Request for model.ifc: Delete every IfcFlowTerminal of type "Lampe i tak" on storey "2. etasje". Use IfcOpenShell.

First a look at what the model holds.

```python
import ifcopenshell
import ifcopenshell.util.element

model = ifcopenshell.open("model.ifc")
print(model.schema)
storey = next(s for s in model.by_type("IfcBuildingStorey") if s.Name == "2. etasje")
terminals = [e for e in ifcopenshell.util.element.get_decomposition(storey) if e.is_a("IfcFlowTerminal")]
seen = {}
for e in terminals:
    element_type = ifcopenshell.util.element.get_type(e)
    name = element_type.Name if element_type not in (None, e) else None
    seen[name] = seen.get(name, 0) + 1
for name, count in sorted(seen.items(), key=str):
    print(count, "x", name)
```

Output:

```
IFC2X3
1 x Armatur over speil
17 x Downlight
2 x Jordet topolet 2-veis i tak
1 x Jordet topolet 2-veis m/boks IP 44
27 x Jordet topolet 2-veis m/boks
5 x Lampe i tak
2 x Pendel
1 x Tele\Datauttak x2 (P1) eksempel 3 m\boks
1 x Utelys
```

```python
import ifcopenshell
import ifcopenshell.api.root
import ifcopenshell.util.element

model = ifcopenshell.open("model.ifc")

storey = next(s for s in model.by_type("IfcBuildingStorey") if s.Name == "2. etasje")
terminals = [e for e in ifcopenshell.util.element.get_decomposition(storey) if e.is_a("IfcFlowTerminal")]
targets = [e for e in terminals if (t := ifcopenshell.util.element.get_type(e)) not in (None, e) and t.Name == "Lampe i tak"]

for e in targets:
    ifcopenshell.api.root.remove_product(model, product=e)
print(len(targets), "removed")

model.write("model_updated.ifc")
```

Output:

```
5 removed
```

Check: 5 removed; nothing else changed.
